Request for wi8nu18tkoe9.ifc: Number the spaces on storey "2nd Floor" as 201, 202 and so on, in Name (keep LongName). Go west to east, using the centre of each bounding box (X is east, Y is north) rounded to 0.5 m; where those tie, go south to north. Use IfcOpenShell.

First a look at what the model holds.

```python
import ifcopenshell
import ifcopenshell.util.element
import ifcopenshell.util.placement

model = ifcopenshell.open("wi8nu18tkoe9.ifc")
print(model.schema)
storey = next(s for s in model.by_type("IfcBuildingStorey") if s.Name == "2nd Floor")
spaces = [e for e in ifcopenshell.util.element.get_decomposition(storey) if e.is_a("IfcSpace")]
for e in sorted(spaces, key=lambda e: e.id()):
    origin = ifcopenshell.util.placement.get_local_placement(e.ObjectPlacement)[:3, 3]
    print(e.id(), e.Name, e.LongName, origin.round(2) + 0.0, sep=" | ")
```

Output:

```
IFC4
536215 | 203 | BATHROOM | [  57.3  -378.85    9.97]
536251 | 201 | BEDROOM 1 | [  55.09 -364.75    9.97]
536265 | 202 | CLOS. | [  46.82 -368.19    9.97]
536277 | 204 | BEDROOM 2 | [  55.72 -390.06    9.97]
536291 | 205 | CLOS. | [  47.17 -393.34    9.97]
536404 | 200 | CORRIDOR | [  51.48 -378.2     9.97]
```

```python
import ifcopenshell
import ifcopenshell.geom
import ifcopenshell.util.element
import ifcopenshell.util.shape

model = ifcopenshell.open("wi8nu18tkoe9.ifc")
settings = ifcopenshell.geom.settings()
settings.set("use-world-coords", True)


def centre(element):
    shape = ifcopenshell.geom.create_shape(settings, element)
    return ifcopenshell.util.shape.get_bbox_centroid(shape.geometry)


storey = next(s for s in model.by_type("IfcBuildingStorey") if s.Name == "2nd Floor")
spaces = [e for e in ifcopenshell.util.element.get_decomposition(storey) if e.is_a("IfcSpace")]

# Insertion points can sit at a corner or the storey origin, so sort by the geometry (in metres).
centres = {e: centre(e) for e in spaces}
spaces.sort(key=lambda e: (round(centres[e][0] / 0.5), centres[e][1]))

for i, e in enumerate(spaces, start=1):
    number = f"2{i:02d}"
    e.Name = number
    print(e.id(), number)

model.write("wi8nu18tkoe9_rev.ifc")
```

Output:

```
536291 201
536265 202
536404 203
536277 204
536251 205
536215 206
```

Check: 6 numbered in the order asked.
